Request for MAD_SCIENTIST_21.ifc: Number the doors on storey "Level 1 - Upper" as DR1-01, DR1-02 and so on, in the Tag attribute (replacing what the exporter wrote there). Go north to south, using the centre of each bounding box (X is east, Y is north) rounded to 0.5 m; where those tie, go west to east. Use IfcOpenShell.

First a look at what the model holds.

```python
import ifcopenshell
import ifcopenshell.util.element
import ifcopenshell.util.placement

model = ifcopenshell.open("MAD_SCIENTIST_21.ifc")
print(model.schema)
storey = next(s for s in model.by_type("IfcBuildingStorey") if s.Name == "Level 1 - Upper")
doors = [e for e in ifcopenshell.util.element.get_decomposition(storey) if e.is_a("IfcDoor")]
for e in sorted(doors, key=lambda e: e.id()):
    origin = ifcopenshell.util.placement.get_local_placement(e.ObjectPlacement)[:3, 3]
    print(e.id(), e.Tag, e.Name, origin.round(2) + 0.0, sep=" | ")
```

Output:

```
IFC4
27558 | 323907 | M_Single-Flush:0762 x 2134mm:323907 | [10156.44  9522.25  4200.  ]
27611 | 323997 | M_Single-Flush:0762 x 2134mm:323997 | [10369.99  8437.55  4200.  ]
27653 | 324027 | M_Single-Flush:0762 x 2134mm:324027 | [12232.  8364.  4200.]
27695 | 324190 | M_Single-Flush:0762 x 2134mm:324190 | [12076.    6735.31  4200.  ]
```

```python
import ifcopenshell
import ifcopenshell.geom
import ifcopenshell.util.element
import ifcopenshell.util.shape

model = ifcopenshell.open("MAD_SCIENTIST_21.ifc")
settings = ifcopenshell.geom.settings()
settings.set("use-world-coords", True)


def centre(element):
    shape = ifcopenshell.geom.create_shape(settings, element)
    return ifcopenshell.util.shape.get_bbox_centroid(shape.geometry)


storey = next(s for s in model.by_type("IfcBuildingStorey") if s.Name == "Level 1 - Upper")
doors = [e for e in ifcopenshell.util.element.get_decomposition(storey) if e.is_a("IfcDoor")]

# Insertion points can sit at a corner or the storey origin, so sort by the geometry (in metres).
centres = {e: centre(e) for e in doors}
doors.sort(key=lambda e: (-round(centres[e][1] / 0.5), centres[e][0]))

for i, e in enumerate(doors, start=1):
    number = f"DR1-{i:02d}"
    e.Tag = number
    print(e.id(), number)

model.write("MAD_SCIENTIST_21_edited.ifc")
```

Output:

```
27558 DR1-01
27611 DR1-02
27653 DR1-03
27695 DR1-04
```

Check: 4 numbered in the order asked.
